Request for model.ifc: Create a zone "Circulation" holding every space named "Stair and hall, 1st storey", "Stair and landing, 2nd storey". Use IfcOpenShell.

First a look at what the model holds.

```python
import ifcopenshell

model = ifcopenshell.open("model.ifc")
print(model.schema)
seen = {}
for space in model.by_type("IfcSpace"):
    seen[space.LongName] = seen.get(space.LongName, 0) + 1
for name, count in sorted(seen.items(), key=str):
    print(count, "x", name)
print("zones:", [z.Name for z in model.by_type("IfcZone")][:20])
```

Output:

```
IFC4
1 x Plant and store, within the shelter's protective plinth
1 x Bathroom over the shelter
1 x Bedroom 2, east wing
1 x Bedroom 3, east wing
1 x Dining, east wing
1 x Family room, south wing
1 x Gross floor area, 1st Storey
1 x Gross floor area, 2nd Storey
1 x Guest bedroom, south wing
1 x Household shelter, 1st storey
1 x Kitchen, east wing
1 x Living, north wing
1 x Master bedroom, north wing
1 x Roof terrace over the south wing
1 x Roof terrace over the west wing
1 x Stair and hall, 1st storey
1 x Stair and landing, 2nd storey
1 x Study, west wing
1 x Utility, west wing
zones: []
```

```python
import ifcopenshell
import ifcopenshell.api.group
import ifcopenshell.api.root

model = ifcopenshell.open("model.ifc")

names = {"Stair and hall, 1st storey", "Stair and landing, 2nd storey"}
spaces = [s for s in model.by_type("IfcSpace") if s.LongName in names]

zone = ifcopenshell.api.root.create_entity(model, ifc_class="IfcZone", name="Circulation")
ifcopenshell.api.group.assign_group(model, products=spaces, group=zone)
print(len(spaces), "spaces in", zone.Name)

model.write("model_edited.ifc")
```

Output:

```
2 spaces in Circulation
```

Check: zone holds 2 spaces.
